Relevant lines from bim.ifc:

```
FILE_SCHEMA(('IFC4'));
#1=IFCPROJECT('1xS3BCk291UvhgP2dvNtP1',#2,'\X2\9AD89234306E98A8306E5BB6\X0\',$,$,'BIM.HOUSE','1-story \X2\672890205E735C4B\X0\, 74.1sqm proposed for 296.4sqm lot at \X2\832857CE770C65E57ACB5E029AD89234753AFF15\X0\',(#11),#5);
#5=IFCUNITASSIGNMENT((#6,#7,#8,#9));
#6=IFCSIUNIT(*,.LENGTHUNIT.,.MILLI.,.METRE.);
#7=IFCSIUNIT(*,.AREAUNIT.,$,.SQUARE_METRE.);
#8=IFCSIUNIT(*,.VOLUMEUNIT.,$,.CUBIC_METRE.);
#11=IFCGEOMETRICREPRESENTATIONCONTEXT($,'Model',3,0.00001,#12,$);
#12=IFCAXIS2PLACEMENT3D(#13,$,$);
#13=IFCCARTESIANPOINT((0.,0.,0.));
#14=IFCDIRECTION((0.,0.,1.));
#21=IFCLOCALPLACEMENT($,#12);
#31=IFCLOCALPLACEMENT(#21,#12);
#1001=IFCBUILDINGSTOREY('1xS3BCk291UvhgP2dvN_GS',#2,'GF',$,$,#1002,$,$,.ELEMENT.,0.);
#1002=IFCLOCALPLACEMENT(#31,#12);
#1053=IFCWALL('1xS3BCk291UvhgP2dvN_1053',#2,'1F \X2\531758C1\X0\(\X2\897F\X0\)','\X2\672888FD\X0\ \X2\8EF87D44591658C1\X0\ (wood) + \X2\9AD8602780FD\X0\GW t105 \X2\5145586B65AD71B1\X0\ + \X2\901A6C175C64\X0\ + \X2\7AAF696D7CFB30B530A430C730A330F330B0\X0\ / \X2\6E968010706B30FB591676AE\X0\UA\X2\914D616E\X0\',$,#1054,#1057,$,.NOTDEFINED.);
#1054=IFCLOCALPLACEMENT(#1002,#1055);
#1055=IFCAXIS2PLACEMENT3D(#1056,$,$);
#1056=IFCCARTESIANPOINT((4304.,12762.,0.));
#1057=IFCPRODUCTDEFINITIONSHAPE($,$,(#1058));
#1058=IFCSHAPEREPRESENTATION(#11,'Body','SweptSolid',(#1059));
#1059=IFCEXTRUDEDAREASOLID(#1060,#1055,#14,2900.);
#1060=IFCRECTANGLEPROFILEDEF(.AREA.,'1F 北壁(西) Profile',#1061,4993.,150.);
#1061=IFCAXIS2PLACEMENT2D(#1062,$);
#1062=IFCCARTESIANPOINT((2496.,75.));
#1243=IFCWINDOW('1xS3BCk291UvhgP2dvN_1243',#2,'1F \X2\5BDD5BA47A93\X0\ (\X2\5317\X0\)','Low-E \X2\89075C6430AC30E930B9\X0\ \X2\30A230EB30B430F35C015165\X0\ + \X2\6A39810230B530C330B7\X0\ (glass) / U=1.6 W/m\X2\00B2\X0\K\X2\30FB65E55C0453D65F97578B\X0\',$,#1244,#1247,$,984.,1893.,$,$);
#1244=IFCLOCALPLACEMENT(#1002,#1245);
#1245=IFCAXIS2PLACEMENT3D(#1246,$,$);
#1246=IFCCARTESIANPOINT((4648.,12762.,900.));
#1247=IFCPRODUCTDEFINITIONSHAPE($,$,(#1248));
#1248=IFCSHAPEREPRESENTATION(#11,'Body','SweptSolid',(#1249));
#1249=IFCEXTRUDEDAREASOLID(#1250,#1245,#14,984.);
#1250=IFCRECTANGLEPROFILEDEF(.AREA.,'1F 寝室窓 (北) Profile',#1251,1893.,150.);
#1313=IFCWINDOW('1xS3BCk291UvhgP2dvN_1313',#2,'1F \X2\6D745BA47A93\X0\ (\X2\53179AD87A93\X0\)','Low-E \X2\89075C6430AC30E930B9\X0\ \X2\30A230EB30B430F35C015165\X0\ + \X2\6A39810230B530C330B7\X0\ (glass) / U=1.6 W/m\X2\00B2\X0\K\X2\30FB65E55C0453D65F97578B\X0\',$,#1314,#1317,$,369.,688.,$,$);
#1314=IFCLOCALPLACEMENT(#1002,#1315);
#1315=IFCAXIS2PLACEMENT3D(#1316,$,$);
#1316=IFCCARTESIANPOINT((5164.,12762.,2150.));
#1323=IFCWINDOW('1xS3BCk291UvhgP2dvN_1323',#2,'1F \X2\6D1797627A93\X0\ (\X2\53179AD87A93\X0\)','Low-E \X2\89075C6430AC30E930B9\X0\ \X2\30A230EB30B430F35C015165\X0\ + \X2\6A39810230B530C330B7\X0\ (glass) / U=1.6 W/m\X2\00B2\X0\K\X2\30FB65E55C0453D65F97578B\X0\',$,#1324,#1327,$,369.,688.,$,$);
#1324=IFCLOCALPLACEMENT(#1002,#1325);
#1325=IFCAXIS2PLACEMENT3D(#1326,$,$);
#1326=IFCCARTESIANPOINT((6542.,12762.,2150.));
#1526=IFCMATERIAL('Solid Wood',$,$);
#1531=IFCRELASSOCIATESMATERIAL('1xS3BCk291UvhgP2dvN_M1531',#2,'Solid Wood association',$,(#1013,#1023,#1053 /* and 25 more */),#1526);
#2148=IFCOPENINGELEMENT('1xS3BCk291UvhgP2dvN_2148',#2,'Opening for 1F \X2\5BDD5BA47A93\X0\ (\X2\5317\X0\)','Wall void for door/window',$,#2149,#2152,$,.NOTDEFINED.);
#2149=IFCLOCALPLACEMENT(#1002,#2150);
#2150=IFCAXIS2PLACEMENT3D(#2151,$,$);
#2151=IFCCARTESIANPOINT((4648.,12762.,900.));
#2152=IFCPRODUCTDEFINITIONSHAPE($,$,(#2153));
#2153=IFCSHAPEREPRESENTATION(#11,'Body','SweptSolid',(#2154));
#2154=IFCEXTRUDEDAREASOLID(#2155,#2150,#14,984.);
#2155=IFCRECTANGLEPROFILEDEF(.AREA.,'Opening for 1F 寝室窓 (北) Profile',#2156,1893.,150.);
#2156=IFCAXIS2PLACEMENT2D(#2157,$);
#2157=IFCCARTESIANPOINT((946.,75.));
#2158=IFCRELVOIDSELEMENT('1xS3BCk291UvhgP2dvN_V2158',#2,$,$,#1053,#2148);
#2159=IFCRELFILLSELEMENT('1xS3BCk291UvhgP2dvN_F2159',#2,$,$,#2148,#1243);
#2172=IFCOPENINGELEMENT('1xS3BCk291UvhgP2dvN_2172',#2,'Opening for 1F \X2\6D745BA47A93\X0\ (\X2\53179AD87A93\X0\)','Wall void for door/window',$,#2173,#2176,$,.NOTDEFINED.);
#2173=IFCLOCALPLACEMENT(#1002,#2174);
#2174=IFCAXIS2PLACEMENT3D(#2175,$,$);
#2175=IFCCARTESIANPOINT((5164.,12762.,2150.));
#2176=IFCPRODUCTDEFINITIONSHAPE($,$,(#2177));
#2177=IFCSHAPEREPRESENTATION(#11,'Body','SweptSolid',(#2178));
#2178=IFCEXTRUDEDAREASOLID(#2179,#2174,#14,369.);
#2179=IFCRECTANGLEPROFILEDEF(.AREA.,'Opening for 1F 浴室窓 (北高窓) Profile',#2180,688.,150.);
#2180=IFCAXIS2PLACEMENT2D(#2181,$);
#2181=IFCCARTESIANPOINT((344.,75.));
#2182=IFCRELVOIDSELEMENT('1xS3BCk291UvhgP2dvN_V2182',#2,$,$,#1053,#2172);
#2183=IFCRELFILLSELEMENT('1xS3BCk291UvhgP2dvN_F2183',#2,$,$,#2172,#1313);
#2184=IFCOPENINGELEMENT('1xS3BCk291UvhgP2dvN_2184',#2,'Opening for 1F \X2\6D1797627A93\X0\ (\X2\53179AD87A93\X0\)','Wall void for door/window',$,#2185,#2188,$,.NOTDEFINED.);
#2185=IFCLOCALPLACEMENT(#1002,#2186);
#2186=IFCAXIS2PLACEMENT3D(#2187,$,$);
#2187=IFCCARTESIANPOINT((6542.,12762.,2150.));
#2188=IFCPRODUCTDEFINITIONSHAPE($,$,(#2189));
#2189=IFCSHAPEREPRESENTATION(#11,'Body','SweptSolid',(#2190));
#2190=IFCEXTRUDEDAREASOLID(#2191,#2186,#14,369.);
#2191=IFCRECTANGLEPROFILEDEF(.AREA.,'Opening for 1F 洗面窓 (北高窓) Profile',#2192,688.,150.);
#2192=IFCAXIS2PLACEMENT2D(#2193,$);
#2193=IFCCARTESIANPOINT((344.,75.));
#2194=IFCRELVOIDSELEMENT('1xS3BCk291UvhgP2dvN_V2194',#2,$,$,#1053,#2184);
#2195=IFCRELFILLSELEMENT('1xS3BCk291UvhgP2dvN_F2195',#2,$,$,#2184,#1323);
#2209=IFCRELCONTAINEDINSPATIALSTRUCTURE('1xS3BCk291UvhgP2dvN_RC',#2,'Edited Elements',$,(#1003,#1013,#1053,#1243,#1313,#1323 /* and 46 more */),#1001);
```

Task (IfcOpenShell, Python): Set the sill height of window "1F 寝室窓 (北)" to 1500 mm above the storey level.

```python
import numpy as np
import ifcopenshell
import ifcopenshell.api.geometry
import ifcopenshell.geom
import ifcopenshell.util.element
import ifcopenshell.util.placement
import ifcopenshell.util.shape
import ifcopenshell.util.unit

model = ifcopenshell.open("bim.ifc")
unit_scale = ifcopenshell.util.unit.calculate_unit_scale(model)

window = model.by_id(1243)
opening = window.FillsVoids[0].RelatingOpeningElement
storey = ifcopenshell.util.element.get_container(window, ifc_class="IfcBuildingStorey")
level = ifcopenshell.util.placement.get_local_placement(storey.ObjectPlacement)[2, 3]

# The opening's origin need not be at the sill, so measure its lowest point.
shape = ifcopenshell.geom.create_shape(ifcopenshell.geom.settings(), opening)
bottom = ifcopenshell.util.shape.get_shape_bottom_elevation(shape, shape.geometry) / unit_scale
dz = level + 1.5 / unit_scale - bottom

shift = np.array([0.0, 0.0, dz])
# The window is not placed relative to its opening, so move both.
for product in (opening, window):
    matrix = ifcopenshell.util.placement.get_local_placement(product.ObjectPlacement)
    matrix[:3, 3] += shift
    ifcopenshell.api.geometry.edit_object_placement(model, product=product, matrix=matrix, is_si=False)

print(f"moved by {dz * unit_scale:+.3f} m")

model.write("bim-out.ifc")
```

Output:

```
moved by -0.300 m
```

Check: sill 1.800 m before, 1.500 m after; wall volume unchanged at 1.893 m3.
